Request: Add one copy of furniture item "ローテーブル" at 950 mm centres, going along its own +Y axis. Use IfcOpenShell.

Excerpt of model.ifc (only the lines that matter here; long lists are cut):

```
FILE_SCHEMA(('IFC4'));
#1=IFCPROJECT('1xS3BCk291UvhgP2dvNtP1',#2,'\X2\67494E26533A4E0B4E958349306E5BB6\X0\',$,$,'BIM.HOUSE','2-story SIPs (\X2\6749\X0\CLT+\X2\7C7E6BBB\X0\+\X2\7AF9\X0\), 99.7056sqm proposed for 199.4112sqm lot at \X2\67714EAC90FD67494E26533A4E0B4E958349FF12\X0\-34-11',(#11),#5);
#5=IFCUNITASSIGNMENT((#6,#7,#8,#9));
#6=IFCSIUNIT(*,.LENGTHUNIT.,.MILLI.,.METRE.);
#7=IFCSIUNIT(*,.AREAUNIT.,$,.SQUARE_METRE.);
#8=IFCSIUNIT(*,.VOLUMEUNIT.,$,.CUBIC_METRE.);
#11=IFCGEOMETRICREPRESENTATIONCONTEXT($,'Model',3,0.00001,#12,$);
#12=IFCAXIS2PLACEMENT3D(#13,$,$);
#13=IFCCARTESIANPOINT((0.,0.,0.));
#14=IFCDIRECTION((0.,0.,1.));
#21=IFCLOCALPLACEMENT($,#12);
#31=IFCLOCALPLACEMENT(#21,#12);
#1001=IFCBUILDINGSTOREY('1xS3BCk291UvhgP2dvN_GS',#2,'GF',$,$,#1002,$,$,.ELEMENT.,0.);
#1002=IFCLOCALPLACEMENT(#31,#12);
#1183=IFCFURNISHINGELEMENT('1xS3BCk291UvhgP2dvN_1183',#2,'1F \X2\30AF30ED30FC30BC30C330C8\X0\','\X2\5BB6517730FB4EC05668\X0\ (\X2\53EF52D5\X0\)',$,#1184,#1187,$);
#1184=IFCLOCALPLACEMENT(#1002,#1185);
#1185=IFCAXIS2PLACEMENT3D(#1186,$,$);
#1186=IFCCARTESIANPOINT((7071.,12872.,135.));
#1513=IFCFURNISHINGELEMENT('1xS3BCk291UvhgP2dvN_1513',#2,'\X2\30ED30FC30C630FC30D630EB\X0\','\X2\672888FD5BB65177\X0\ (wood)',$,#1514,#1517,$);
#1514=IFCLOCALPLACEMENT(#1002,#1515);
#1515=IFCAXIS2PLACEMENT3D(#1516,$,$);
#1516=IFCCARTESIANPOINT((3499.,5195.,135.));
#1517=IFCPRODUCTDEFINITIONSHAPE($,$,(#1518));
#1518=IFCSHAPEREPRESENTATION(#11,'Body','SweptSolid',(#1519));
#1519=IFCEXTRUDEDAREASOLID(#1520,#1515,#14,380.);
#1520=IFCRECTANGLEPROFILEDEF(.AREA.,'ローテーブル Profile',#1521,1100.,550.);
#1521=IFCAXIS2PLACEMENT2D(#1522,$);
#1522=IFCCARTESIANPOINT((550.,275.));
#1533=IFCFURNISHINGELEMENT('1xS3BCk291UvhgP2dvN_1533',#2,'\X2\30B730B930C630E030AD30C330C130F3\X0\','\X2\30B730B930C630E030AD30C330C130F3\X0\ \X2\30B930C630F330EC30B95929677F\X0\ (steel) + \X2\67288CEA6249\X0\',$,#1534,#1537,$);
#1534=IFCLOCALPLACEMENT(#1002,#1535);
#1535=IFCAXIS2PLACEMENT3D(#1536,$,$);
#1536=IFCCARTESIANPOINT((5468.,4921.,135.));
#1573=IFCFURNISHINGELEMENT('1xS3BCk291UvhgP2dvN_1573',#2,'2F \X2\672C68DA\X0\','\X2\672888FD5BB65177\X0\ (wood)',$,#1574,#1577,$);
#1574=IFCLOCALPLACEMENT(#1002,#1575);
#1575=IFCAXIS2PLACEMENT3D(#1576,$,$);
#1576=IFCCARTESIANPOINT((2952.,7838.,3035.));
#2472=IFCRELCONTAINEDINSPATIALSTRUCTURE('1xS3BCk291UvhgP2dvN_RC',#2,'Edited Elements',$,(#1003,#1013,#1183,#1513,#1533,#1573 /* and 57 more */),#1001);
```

```python
import ifcopenshell
import ifcopenshell.api.geometry
import ifcopenshell.api.root
import ifcopenshell.util.element
import ifcopenshell.util.placement

model = ifcopenshell.open("model.ifc")


def reuse_history(source, copy):
    """copy_class also copies each property set's owner history, people and application; keep the originals."""
    for rel in copy.IsDefinedBy:
        if rel.is_a("IfcRelDefinesByProperties") and (history := rel.RelatingPropertyDefinition.OwnerHistory):
            rel.RelatingPropertyDefinition.OwnerHistory = source.OwnerHistory
            ifcopenshell.util.element.remove_deep2(model, history)


source = model.by_id(1513)
base = ifcopenshell.util.placement.get_local_placement(source.ObjectPlacement)
step = base[:3, 1] * 950.0

for i in range(1, 2):
    copy = ifcopenshell.api.root.copy_class(model, product=source)
    copy.Representation = ifcopenshell.util.element.copy_deep(
        model, source.Representation, exclude=["IfcGeometricRepresentationContext", "IfcRepresentationMap"]
    )
    reuse_history(source, copy)
    matrix = base.copy()
    matrix[:3, 3] += i * step
    print("added at", matrix[:3, 3].round(3) + 0.0)
    ifcopenshell.api.geometry.edit_object_placement(model, product=copy, matrix=matrix, is_si=False)

model.write("model-out.ifc")
```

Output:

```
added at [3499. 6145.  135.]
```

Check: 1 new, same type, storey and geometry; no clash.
